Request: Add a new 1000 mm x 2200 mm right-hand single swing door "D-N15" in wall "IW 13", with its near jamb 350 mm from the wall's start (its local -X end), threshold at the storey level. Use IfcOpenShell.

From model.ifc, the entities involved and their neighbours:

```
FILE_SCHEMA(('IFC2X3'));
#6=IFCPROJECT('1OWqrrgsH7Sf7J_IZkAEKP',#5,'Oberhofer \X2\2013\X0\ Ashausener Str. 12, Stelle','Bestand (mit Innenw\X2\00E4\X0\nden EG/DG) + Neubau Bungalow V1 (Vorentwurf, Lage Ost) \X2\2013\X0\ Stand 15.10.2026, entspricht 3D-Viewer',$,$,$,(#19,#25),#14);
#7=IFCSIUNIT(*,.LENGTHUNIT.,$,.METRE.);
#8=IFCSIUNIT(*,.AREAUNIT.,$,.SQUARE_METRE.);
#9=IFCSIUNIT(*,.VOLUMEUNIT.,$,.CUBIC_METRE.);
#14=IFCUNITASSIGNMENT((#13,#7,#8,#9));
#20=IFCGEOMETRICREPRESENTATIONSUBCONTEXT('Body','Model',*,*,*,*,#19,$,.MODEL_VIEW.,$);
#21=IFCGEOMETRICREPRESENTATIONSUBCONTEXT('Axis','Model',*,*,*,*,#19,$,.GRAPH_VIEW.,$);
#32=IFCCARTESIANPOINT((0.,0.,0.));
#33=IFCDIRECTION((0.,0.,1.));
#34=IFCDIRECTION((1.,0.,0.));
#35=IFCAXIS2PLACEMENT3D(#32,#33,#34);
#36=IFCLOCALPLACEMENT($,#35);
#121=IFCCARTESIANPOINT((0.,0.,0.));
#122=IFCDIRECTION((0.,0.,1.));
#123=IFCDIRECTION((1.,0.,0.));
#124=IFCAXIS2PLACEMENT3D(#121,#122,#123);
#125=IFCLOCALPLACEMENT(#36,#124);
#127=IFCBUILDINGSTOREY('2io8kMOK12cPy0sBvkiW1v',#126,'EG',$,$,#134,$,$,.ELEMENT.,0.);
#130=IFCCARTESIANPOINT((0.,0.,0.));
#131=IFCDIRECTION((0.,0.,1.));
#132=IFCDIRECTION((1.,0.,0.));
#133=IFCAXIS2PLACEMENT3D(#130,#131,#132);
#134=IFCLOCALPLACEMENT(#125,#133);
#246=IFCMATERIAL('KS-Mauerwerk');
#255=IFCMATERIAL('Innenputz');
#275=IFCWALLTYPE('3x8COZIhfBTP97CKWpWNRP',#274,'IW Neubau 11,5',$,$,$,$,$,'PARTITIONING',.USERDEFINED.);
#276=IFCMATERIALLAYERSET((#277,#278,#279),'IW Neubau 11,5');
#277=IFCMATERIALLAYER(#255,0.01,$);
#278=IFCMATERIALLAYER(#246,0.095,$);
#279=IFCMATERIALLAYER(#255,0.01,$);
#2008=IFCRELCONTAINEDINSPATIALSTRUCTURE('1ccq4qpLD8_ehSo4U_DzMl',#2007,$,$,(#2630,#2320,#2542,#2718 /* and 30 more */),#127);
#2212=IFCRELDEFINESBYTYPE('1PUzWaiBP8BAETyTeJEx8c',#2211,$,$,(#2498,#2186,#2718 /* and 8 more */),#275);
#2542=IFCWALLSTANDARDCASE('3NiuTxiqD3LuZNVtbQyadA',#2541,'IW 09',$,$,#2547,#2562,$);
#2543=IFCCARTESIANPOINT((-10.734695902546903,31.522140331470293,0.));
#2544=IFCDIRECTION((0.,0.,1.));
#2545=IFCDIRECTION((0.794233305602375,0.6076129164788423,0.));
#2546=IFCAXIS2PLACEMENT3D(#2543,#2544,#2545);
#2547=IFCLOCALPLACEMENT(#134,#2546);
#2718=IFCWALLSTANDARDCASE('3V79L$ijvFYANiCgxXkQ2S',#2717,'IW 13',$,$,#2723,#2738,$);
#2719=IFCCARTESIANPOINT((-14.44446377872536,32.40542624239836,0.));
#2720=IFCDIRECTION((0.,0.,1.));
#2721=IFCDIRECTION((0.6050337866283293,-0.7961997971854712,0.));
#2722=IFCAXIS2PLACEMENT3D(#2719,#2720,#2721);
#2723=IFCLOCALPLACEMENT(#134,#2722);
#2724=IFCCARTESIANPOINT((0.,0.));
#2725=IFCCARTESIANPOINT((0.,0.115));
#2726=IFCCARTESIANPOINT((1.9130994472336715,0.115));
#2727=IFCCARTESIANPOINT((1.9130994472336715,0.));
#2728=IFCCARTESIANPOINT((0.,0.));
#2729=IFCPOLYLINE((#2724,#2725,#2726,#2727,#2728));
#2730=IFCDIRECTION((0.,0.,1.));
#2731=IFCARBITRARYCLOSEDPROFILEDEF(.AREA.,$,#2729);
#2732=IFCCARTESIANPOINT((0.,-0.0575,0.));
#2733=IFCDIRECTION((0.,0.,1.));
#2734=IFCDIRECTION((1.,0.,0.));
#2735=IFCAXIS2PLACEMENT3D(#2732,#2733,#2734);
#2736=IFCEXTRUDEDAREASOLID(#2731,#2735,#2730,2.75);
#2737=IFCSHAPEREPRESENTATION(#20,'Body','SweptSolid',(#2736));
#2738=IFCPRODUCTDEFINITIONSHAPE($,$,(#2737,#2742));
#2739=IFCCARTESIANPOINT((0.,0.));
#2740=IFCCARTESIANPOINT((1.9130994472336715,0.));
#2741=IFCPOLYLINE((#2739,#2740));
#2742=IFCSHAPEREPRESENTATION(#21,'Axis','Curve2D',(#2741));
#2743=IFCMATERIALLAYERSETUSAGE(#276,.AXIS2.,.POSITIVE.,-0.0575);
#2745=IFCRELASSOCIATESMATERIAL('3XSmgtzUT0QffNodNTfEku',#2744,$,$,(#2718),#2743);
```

```python
import numpy as np
import ifcopenshell
import ifcopenshell.api.feature
import ifcopenshell.api.geometry
import ifcopenshell.api.root
import ifcopenshell.api.spatial
import ifcopenshell.api.type
import ifcopenshell.geom
import ifcopenshell.util.element
import ifcopenshell.util.placement
import ifcopenshell.util.representation
import ifcopenshell.util.shape
import ifcopenshell.util.unit

model = ifcopenshell.open("model.ifc")
unit_scale = ifcopenshell.util.unit.calculate_unit_scale(model)
settings = ifcopenshell.geom.settings()


def volume(element):
    """Net volume in cubic metres, openings subtracted."""
    shape = ifcopenshell.geom.create_shape(settings, element)
    return ifcopenshell.util.shape.get_volume(shape.geometry)


wall = model.by_id(2718)
storey = ifcopenshell.util.element.get_container(wall, ifc_class="IfcBuildingStorey")
context = ifcopenshell.util.representation.get_context(model, "Model", "Body", "MODEL_VIEW")
before = volume(wall)

width, height, from_end, sill = 1, 2.2, 0.35, 0.0  # metres

# The wall runs along its own X axis, and the end named is its -X end.
wall_shape = ifcopenshell.geom.create_shape(settings, wall)
x, y, z = ifcopenshell.util.shape.get_vertices(wall_shape.geometry).T
start = x.min() + from_end
face, thickness = float(y.min()), float(y.max() - y.min())
wall_matrix = ifcopenshell.util.placement.get_local_placement(wall.ObjectPlacement)
level = ifcopenshell.util.placement.get_local_placement(storey.ObjectPlacement)[2, 3]


def in_wall(x, y):
    """Placement at x, y metres in the wall's axes, at sill height."""
    matrix = wall_matrix.copy()
    matrix[:, 3] = wall_matrix @ np.array([x / unit_scale, y / unit_scale, 0.0, 1.0])
    matrix[2, 3] = level + sill / unit_scale
    return matrix


# Opening: a box that overshoots both wall faces by 50 mm.
opening = ifcopenshell.api.root.create_entity(model, ifc_class="IfcOpeningElement")
box = ifcopenshell.api.geometry.add_wall_representation(
    model, context=context, length=width, height=height, thickness=thickness + 0.1
)
ifcopenshell.api.geometry.assign_representation(model, product=opening, representation=box)
ifcopenshell.api.geometry.edit_object_placement(model, product=opening, matrix=in_wall(start, face - 0.05), is_si=False)
ifcopenshell.api.feature.add_feature(model, feature=opening, element=wall)

door = ifcopenshell.api.root.create_entity(model, ifc_class="IfcDoor", name="D-N15")
door.OverallWidth, door.OverallHeight = width / unit_scale, height / unit_scale
body = ifcopenshell.api.geometry.add_door_representation(
    model,
    context=context,
    overall_width=door.OverallWidth,
    overall_height=door.OverallHeight,
    operation_type="SINGLE_SWING_RIGHT",
    lining_properties={"LiningDepth": thickness / unit_scale, "ThresholdDepth": thickness / unit_scale},
)
ifcopenshell.api.geometry.assign_representation(model, product=door, representation=body)
ifcopenshell.api.spatial.assign_container(model, products=[door], relating_structure=storey)
fills = ifcopenshell.api.feature.add_filling(model, opening=opening, element=door)
fills.OwnerHistory = door.OwnerHistory  # required in IFC2X3

# IFC2X3 keeps the operation on the door style.
style = ifcopenshell.api.root.create_entity(model, ifc_class="IfcDoorStyle", name="D-N15")
style.OperationType, style.ConstructionType = "SINGLE_SWING_RIGHT", "NOTDEFINED"
style.ParameterTakesPrecedence = style.Sizeable = False
ifcopenshell.api.type.assign_type(model, related_objects=[door], relating_type=style)

# The lining spans the wall, so the door starts at the wall face.
ifcopenshell.api.geometry.edit_object_placement(model, product=door, matrix=in_wall(start, face), is_si=False)

after = volume(wall)

print(f"wall volume {before:.3f} -> {after:.3f} m3")

model.write("model_edited.ifc")
```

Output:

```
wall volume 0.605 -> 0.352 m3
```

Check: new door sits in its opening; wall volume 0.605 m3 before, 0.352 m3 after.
